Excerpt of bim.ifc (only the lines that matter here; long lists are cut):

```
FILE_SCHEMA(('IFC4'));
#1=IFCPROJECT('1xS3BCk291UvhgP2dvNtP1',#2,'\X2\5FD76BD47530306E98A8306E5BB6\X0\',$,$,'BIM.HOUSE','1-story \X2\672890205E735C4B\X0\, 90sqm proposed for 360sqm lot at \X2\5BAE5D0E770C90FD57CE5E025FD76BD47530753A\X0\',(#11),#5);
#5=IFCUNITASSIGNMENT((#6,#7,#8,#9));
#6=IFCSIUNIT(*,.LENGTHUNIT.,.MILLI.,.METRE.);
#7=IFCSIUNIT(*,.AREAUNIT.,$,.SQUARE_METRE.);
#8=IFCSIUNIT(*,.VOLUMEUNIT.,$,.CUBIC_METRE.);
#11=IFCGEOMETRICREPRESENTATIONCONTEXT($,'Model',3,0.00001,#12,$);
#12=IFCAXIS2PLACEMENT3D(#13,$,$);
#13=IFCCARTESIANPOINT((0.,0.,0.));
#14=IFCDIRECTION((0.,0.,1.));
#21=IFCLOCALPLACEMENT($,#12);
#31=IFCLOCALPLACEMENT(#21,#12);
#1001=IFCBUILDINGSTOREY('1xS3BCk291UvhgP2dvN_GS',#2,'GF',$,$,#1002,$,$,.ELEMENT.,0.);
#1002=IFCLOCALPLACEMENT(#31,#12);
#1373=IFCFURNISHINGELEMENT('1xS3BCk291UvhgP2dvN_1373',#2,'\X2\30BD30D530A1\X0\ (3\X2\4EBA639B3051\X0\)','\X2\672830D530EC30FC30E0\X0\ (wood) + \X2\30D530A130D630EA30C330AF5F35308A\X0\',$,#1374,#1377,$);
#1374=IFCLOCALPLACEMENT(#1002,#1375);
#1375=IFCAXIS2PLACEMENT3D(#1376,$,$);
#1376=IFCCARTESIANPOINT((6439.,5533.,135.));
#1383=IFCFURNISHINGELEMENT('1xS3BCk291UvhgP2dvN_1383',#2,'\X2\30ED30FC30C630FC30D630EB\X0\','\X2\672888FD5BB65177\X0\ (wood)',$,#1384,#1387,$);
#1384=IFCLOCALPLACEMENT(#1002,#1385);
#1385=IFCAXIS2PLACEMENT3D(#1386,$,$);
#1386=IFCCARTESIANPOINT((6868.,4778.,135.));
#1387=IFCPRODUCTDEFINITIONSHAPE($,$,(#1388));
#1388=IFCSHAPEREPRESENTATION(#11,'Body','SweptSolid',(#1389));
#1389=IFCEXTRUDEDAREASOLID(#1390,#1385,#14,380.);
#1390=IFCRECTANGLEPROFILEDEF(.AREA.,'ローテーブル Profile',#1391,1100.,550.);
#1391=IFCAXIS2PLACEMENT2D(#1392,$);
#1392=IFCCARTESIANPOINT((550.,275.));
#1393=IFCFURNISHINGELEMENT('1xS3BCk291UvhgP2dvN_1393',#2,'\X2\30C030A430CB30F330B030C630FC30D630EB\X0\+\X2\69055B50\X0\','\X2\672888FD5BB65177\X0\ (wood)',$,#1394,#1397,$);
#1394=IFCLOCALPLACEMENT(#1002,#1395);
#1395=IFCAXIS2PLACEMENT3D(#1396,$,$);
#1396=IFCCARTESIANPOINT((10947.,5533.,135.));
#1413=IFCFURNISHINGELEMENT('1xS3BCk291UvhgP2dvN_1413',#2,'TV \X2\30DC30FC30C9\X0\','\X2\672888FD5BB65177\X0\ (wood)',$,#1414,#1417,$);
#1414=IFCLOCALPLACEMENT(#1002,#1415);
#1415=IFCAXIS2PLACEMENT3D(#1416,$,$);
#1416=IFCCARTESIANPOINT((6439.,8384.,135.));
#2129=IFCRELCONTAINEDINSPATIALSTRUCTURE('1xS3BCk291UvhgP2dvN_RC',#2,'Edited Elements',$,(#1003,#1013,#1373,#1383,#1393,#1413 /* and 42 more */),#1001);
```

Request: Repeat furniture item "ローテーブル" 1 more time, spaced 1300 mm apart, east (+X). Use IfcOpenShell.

```python
import numpy as np
import ifcopenshell
import ifcopenshell.api.geometry
import ifcopenshell.api.root
import ifcopenshell.util.element
import ifcopenshell.util.placement
import ifcopenshell.util.unit

model = ifcopenshell.open("bim.ifc")
unit_scale = ifcopenshell.util.unit.calculate_unit_scale(model)


def reuse_history(source, copy):
    """copy_class also copies each property set's owner history, people and application; keep the originals."""
    for rel in copy.IsDefinedBy:
        if rel.is_a("IfcRelDefinesByProperties") and (history := rel.RelatingPropertyDefinition.OwnerHistory):
            rel.RelatingPropertyDefinition.OwnerHistory = source.OwnerHistory
            ifcopenshell.util.element.remove_deep2(model, history)


source = model.by_guid("1xS3BCk291UvhgP2dvN_1383")
base = ifcopenshell.util.placement.get_local_placement(source.ObjectPlacement)
step = np.array([1.0, 0.0, 0.0]) * 1.3 / unit_scale

for i in range(1, 2):
    copy = ifcopenshell.api.root.copy_class(model, product=source)
    copy.Representation = ifcopenshell.util.element.copy_deep(
        model, source.Representation, exclude=["IfcGeometricRepresentationContext", "IfcRepresentationMap"]
    )
    reuse_history(source, copy)
    matrix = base.copy()
    matrix[:3, 3] += i * step
    print("added at", matrix[:3, 3].round(3) + 0.0)
    ifcopenshell.api.geometry.edit_object_placement(model, product=copy, matrix=matrix, is_si=False)

model.write("bim_v2.ifc")
```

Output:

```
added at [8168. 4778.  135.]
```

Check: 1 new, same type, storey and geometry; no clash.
